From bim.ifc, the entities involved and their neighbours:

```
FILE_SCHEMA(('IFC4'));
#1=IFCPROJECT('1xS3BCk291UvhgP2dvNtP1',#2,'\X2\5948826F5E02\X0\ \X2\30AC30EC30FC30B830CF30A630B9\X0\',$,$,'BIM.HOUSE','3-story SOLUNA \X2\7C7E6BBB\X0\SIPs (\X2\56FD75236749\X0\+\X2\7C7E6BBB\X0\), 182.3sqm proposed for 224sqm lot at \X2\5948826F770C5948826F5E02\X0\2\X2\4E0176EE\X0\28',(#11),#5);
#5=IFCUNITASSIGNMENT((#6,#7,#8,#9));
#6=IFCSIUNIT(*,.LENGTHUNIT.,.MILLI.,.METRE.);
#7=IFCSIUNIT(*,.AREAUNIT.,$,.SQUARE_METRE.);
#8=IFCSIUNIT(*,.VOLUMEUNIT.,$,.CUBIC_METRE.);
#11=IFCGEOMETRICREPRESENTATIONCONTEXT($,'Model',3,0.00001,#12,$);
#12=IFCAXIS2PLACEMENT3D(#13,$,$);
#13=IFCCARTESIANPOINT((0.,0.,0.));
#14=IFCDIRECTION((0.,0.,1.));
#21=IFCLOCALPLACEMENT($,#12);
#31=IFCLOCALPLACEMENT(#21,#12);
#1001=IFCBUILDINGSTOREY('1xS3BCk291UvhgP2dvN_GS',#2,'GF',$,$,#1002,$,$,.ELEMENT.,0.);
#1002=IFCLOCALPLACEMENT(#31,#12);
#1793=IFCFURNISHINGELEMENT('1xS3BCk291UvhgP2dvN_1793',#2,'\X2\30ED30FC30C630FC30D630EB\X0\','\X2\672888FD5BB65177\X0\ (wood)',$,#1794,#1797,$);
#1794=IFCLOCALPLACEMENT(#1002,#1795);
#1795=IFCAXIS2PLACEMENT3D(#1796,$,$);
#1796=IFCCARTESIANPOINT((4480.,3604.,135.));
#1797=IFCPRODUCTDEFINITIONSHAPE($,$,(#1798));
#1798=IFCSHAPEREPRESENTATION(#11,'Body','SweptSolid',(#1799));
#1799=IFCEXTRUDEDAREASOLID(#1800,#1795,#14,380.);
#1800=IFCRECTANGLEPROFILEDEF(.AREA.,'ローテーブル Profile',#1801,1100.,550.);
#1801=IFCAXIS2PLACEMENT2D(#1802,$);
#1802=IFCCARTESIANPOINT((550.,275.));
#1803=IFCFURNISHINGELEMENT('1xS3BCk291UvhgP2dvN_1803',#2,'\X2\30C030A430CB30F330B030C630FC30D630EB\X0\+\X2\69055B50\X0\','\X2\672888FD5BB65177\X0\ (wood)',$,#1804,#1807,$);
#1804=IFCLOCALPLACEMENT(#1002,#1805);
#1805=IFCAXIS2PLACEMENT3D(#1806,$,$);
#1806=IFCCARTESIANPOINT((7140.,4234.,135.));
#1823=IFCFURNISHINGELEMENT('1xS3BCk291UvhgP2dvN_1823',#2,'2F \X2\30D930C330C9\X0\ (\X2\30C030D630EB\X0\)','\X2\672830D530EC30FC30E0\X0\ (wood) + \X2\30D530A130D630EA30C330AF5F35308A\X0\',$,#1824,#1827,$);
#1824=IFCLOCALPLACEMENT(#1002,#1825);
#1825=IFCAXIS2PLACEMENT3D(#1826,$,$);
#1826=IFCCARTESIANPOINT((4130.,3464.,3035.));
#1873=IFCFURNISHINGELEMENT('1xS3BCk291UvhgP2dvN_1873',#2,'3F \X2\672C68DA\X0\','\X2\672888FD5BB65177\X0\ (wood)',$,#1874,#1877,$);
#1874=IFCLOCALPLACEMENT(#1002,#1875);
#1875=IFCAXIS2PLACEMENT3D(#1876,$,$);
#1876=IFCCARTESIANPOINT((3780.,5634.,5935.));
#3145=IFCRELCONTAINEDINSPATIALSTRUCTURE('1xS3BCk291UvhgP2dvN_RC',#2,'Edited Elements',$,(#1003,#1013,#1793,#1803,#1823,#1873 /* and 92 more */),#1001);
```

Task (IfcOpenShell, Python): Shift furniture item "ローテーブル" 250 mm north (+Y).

```python
import ifcopenshell
import ifcopenshell.api.geometry
import ifcopenshell.util.placement

model = ifcopenshell.open("bim.ifc")

item = model.by_id(1793)
matrix = ifcopenshell.util.placement.get_local_placement(item.ObjectPlacement)
matrix[1, 3] += 250.0
ifcopenshell.api.geometry.edit_object_placement(model, product=item, matrix=matrix, is_si=False)

print(ifcopenshell.util.placement.get_local_placement(item.ObjectPlacement).round(3) + 0.0)

model.write("bim_rev.ifc")
```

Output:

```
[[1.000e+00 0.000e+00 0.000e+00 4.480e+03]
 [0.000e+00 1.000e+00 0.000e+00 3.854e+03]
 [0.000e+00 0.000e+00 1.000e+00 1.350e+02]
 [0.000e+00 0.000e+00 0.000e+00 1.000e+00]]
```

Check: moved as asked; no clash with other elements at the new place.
